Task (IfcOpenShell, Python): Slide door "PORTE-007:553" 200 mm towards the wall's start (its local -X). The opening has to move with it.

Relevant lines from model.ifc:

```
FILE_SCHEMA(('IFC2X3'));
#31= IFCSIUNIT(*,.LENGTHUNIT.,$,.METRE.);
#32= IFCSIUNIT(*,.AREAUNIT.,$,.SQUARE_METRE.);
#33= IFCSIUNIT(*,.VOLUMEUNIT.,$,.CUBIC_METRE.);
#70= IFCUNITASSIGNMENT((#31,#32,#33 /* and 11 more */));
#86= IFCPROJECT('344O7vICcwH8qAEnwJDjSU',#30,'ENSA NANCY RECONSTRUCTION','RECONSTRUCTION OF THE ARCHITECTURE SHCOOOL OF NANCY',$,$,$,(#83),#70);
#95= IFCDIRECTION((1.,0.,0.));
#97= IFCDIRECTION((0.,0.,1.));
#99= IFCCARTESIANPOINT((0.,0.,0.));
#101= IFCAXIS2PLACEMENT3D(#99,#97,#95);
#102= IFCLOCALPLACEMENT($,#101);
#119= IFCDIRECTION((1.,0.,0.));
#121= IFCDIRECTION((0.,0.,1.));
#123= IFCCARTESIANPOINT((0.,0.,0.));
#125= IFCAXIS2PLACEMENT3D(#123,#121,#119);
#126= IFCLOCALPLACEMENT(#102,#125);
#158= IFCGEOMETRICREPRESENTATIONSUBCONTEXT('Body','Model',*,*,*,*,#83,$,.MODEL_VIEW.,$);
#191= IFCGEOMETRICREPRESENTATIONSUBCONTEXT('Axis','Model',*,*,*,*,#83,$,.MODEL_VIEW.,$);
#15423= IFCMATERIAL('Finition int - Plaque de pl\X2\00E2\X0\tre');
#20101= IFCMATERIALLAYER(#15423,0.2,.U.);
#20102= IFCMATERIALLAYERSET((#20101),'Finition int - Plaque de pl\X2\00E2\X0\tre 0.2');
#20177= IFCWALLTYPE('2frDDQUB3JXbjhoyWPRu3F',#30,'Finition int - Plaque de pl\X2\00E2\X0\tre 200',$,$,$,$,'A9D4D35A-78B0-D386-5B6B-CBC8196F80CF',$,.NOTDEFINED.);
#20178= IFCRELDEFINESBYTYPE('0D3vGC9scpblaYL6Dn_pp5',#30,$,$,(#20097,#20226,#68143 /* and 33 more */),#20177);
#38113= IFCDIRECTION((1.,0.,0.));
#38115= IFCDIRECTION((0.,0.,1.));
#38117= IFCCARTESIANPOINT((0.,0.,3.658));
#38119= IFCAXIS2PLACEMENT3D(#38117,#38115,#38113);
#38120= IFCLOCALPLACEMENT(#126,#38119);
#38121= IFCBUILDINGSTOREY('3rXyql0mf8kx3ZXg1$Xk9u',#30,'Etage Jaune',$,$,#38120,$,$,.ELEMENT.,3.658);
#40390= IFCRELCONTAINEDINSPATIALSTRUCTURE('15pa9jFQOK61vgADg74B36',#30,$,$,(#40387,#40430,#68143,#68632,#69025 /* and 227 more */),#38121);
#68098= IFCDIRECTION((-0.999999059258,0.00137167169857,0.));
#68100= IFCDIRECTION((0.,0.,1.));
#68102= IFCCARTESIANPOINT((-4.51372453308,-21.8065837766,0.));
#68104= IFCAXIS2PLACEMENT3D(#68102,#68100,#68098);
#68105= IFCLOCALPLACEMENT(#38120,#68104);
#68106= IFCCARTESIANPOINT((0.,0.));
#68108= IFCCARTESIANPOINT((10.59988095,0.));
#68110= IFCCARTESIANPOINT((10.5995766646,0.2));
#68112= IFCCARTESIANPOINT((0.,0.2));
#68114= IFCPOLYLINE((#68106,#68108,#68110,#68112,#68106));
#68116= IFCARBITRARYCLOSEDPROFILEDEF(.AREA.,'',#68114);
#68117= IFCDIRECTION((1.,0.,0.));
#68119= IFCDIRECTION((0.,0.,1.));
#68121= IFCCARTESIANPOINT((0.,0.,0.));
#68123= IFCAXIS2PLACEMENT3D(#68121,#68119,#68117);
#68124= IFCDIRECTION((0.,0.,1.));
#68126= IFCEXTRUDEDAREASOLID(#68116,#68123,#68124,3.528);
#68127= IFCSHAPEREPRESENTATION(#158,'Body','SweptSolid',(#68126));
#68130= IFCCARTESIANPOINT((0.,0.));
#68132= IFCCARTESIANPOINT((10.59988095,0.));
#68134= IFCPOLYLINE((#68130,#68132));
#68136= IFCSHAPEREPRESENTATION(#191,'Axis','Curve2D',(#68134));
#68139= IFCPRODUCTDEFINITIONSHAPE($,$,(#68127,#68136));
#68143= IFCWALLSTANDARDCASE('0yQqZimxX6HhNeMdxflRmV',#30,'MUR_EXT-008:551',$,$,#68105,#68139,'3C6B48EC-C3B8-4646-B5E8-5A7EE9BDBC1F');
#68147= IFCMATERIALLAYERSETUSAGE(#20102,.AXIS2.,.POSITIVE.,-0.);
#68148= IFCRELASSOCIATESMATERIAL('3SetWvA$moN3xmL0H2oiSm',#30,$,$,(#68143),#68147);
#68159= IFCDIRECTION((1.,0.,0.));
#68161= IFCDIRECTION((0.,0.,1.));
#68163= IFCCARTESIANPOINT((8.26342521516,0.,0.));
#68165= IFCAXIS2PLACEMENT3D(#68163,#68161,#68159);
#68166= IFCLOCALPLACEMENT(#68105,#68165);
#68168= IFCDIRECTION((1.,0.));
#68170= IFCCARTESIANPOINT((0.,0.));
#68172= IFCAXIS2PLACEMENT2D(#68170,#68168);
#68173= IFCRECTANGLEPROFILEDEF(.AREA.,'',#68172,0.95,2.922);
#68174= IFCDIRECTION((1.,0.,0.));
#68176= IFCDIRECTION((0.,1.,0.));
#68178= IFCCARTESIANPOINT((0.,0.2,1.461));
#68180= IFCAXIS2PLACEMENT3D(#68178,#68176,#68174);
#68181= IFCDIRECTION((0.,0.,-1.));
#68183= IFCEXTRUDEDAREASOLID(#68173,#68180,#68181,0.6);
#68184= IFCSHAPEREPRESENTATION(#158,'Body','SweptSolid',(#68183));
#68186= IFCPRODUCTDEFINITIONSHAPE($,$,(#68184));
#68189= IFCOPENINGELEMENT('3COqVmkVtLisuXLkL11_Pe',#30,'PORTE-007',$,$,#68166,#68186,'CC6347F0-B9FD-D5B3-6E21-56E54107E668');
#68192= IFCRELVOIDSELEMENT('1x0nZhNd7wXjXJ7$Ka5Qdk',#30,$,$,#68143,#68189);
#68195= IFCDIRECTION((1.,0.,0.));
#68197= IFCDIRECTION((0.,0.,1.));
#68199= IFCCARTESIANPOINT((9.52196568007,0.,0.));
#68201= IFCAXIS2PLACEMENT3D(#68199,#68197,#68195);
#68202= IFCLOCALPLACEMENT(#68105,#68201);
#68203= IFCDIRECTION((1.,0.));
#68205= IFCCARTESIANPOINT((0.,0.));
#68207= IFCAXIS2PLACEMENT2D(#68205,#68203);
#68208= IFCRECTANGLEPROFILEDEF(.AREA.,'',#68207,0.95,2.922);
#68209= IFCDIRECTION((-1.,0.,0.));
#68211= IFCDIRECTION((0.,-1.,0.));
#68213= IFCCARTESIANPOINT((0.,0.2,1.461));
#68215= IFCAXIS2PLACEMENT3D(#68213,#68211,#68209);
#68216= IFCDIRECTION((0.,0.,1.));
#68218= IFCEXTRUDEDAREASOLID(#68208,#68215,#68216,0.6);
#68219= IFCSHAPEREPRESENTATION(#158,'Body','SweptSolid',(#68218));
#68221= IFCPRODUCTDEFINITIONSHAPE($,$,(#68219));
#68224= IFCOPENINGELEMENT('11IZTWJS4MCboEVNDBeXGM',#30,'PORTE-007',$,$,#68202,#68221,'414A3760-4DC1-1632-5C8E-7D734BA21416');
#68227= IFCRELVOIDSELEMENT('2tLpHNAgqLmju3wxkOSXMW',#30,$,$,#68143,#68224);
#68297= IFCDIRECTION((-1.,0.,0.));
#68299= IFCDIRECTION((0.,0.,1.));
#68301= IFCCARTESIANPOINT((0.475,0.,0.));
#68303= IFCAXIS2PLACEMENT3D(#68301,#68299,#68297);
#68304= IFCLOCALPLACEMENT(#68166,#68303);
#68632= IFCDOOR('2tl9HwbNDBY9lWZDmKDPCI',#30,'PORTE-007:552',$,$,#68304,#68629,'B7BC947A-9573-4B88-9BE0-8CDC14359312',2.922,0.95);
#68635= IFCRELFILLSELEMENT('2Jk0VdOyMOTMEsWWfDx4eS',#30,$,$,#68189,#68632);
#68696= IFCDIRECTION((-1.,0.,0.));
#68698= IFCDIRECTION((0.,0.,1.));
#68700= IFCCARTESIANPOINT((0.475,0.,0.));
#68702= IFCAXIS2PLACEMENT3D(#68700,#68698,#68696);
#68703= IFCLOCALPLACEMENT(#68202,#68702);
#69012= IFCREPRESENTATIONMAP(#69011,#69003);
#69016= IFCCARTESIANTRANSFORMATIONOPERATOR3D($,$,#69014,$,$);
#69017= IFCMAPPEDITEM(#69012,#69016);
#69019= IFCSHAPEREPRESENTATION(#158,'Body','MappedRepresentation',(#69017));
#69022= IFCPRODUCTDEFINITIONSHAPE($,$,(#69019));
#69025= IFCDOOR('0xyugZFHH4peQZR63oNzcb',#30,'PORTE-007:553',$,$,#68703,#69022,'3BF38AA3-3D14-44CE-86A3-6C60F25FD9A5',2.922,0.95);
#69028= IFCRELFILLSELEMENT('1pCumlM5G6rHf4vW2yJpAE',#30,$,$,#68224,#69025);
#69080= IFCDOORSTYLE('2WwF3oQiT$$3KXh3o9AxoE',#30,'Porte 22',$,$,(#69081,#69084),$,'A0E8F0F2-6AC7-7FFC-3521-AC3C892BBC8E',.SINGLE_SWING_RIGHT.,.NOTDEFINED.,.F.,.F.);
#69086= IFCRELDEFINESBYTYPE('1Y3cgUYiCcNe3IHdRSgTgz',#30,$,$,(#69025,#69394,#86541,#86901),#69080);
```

```python
import ifcopenshell
import ifcopenshell.api.geometry
import ifcopenshell.util.placement
import ifcopenshell.util.unit

model = ifcopenshell.open("model.ifc")
unit_scale = ifcopenshell.util.unit.calculate_unit_scale(model)

door = model.by_id(69025)
opening = door.FillsVoids[0].RelatingOpeningElement
wall = opening.VoidsElements[0].RelatingBuildingElement

wall_matrix = ifcopenshell.util.placement.get_local_placement(wall.ObjectPlacement)
shift = wall_matrix[:3, 0] * -0.2 / unit_scale
before = ifcopenshell.util.placement.get_local_placement(door.ObjectPlacement)[:3, 3].copy()

# The door is placed relative to its opening, so it follows when the opening moves.
matrix = ifcopenshell.util.placement.get_local_placement(opening.ObjectPlacement)
matrix[:3, 3] += shift
ifcopenshell.api.geometry.edit_object_placement(
    model, product=opening, matrix=matrix, is_si=False, should_transform_children=True
)

after = ifcopenshell.util.placement.get_local_placement(door.ObjectPlacement)[:3, 3]
print("door moved by", (after - before).round(3) + 0.0)

model.write("model_updated.ifc")
```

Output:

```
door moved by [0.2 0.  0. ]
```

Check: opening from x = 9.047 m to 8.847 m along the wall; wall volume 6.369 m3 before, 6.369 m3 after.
